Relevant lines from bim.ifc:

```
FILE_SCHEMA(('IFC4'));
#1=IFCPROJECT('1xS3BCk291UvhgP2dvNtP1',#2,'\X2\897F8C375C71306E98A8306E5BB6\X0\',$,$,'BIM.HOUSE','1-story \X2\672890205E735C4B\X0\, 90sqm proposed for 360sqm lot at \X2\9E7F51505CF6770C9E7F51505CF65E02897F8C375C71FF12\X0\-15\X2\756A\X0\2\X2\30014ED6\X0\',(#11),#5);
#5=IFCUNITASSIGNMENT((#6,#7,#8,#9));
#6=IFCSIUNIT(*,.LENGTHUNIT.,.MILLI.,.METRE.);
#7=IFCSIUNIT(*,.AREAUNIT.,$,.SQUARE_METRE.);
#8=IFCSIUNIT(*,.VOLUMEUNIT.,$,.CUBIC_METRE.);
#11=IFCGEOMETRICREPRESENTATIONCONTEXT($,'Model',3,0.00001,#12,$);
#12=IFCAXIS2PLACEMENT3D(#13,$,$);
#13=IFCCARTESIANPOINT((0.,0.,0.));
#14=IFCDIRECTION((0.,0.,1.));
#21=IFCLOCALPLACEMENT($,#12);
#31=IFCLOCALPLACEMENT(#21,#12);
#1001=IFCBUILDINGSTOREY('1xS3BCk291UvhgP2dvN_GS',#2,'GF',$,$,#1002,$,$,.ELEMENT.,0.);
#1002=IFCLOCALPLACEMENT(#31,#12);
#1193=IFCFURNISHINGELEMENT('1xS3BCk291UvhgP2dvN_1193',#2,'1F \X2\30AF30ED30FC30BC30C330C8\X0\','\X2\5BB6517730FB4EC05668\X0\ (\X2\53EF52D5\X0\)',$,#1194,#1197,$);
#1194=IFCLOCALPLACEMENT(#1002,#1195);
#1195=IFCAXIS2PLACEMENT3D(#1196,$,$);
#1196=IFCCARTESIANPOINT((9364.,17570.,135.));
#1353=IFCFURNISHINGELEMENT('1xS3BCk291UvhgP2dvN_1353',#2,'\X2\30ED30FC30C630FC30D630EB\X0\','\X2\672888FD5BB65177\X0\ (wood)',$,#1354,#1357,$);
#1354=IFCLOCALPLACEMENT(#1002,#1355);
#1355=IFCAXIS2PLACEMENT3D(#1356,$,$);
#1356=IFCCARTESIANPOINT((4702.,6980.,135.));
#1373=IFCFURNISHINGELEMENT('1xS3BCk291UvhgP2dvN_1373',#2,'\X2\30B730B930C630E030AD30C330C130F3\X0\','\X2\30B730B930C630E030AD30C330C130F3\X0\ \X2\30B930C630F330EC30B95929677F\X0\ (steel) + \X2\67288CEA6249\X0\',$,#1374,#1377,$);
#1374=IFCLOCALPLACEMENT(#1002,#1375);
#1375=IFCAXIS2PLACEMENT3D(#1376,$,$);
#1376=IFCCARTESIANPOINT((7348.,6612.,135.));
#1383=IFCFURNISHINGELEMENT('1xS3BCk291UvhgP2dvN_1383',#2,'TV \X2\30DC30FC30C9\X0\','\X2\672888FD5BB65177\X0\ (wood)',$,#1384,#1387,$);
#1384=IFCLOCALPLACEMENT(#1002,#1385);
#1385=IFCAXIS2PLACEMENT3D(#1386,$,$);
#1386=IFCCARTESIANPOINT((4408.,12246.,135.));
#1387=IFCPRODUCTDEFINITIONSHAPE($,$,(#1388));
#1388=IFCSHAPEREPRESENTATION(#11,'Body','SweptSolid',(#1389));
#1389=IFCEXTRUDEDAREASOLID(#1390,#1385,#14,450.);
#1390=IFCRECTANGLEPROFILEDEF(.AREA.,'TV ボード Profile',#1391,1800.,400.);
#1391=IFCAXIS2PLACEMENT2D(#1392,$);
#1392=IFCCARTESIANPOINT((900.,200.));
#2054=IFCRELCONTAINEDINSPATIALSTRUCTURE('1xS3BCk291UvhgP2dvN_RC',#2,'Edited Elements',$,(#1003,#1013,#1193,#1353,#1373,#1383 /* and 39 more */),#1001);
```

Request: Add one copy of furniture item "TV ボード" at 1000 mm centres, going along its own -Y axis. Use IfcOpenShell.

```python
import ifcopenshell
import ifcopenshell.api.geometry
import ifcopenshell.api.root
import ifcopenshell.util.element
import ifcopenshell.util.placement
import ifcopenshell.util.unit

model = ifcopenshell.open("bim.ifc")
unit_scale = ifcopenshell.util.unit.calculate_unit_scale(model)


def reuse_history(source, copy):
    """copy_class also copies each property set's owner history, people and application; keep the originals."""
    for rel in copy.IsDefinedBy:
        if rel.is_a("IfcRelDefinesByProperties") and (history := rel.RelatingPropertyDefinition.OwnerHistory):
            rel.RelatingPropertyDefinition.OwnerHistory = source.OwnerHistory
            ifcopenshell.util.element.remove_deep2(model, history)


source = model.by_guid("1xS3BCk291UvhgP2dvN_1383")
base = ifcopenshell.util.placement.get_local_placement(source.ObjectPlacement)
step = -base[:3, 1] * 1 / unit_scale

for i in range(1, 2):
    copy = ifcopenshell.api.root.copy_class(model, product=source)
    copy.Representation = ifcopenshell.util.element.copy_deep(
        model, source.Representation, exclude=["IfcGeometricRepresentationContext", "IfcRepresentationMap"]
    )
    reuse_history(source, copy)
    matrix = base.copy()
    matrix[:3, 3] += i * step
    print("added at", matrix[:3, 3].round(3) + 0.0)
    ifcopenshell.api.geometry.edit_object_placement(model, product=copy, matrix=matrix, is_si=False)

model.write("bim_v2.ifc")
```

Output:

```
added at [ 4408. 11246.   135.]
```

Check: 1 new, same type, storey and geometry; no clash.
